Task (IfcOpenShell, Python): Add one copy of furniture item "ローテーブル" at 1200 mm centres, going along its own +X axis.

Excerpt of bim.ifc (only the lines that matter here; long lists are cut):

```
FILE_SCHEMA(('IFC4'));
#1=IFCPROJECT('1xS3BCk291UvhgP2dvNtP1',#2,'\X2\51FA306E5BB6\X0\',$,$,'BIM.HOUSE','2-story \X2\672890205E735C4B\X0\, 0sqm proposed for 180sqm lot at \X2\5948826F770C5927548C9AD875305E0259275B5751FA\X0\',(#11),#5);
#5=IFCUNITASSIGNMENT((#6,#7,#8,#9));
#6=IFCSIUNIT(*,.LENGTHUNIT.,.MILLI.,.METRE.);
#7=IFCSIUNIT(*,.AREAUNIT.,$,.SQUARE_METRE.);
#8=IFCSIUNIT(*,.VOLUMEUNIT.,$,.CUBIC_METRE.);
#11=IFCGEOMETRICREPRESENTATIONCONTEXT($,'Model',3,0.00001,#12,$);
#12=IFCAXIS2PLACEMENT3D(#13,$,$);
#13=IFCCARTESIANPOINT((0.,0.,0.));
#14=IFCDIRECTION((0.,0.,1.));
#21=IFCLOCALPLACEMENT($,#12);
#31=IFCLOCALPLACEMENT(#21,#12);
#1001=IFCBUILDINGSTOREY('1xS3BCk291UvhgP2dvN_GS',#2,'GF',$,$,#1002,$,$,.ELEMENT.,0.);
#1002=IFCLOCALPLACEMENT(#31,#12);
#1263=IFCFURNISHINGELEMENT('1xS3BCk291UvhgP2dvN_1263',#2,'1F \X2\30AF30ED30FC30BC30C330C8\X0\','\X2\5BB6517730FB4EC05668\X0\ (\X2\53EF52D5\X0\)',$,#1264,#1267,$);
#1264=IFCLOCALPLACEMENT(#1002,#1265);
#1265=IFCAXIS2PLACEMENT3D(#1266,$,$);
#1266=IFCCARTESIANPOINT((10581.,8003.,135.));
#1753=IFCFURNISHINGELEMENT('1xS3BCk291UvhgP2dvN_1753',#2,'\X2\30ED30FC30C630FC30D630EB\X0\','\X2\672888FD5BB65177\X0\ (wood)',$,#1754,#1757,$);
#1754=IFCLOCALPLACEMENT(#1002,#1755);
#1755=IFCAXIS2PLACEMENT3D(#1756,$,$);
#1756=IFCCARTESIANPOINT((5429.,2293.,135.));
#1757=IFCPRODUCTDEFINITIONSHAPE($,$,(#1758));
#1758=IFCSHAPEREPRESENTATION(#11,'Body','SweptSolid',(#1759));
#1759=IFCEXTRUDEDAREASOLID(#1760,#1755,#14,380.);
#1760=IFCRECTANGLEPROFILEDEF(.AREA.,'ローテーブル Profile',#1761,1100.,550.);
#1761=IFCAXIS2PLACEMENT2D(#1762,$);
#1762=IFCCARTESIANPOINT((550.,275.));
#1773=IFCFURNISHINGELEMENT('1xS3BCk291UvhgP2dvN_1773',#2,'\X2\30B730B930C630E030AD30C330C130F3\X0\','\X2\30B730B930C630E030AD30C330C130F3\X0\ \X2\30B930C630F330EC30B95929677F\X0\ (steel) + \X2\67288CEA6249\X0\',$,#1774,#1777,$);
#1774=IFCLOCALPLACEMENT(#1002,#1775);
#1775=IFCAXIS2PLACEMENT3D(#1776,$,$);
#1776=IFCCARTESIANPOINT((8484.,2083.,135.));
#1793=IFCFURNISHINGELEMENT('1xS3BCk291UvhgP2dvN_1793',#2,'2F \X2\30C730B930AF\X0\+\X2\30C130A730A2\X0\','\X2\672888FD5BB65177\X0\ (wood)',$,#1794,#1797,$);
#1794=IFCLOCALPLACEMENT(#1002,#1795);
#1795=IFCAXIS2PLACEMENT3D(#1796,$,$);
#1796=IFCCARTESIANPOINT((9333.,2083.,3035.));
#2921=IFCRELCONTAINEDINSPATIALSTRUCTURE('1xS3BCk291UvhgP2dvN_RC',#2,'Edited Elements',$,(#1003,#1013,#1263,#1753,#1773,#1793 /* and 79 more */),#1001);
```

```python
import ifcopenshell
import ifcopenshell.api.geometry
import ifcopenshell.api.root
import ifcopenshell.util.element
import ifcopenshell.util.placement
import ifcopenshell.util.unit

model = ifcopenshell.open("bim.ifc")
unit_scale = ifcopenshell.util.unit.calculate_unit_scale(model)


def reuse_history(source, copy):
    """copy_class also copies each property set's owner history, people and application; keep the originals."""
    for rel in copy.IsDefinedBy:
        if rel.is_a("IfcRelDefinesByProperties") and (history := rel.RelatingPropertyDefinition.OwnerHistory):
            rel.RelatingPropertyDefinition.OwnerHistory = source.OwnerHistory
            ifcopenshell.util.element.remove_deep2(model, history)


source = model.by_guid("1xS3BCk291UvhgP2dvN_1753")
base = ifcopenshell.util.placement.get_local_placement(source.ObjectPlacement)
step = base[:3, 0] * 1.2 / unit_scale

for i in range(1, 2):
    copy = ifcopenshell.api.root.copy_class(model, product=source)
    copy.Representation = ifcopenshell.util.element.copy_deep(
        model, source.Representation, exclude=["IfcGeometricRepresentationContext", "IfcRepresentationMap"]
    )
    reuse_history(source, copy)
    matrix = base.copy()
    matrix[:3, 3] += i * step
    print("added at", matrix[:3, 3].round(3) + 0.0)
    ifcopenshell.api.geometry.edit_object_placement(model, product=copy, matrix=matrix, is_si=False)

model.write("bim-out.ifc")
```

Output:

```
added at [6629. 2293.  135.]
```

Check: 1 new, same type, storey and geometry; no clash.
